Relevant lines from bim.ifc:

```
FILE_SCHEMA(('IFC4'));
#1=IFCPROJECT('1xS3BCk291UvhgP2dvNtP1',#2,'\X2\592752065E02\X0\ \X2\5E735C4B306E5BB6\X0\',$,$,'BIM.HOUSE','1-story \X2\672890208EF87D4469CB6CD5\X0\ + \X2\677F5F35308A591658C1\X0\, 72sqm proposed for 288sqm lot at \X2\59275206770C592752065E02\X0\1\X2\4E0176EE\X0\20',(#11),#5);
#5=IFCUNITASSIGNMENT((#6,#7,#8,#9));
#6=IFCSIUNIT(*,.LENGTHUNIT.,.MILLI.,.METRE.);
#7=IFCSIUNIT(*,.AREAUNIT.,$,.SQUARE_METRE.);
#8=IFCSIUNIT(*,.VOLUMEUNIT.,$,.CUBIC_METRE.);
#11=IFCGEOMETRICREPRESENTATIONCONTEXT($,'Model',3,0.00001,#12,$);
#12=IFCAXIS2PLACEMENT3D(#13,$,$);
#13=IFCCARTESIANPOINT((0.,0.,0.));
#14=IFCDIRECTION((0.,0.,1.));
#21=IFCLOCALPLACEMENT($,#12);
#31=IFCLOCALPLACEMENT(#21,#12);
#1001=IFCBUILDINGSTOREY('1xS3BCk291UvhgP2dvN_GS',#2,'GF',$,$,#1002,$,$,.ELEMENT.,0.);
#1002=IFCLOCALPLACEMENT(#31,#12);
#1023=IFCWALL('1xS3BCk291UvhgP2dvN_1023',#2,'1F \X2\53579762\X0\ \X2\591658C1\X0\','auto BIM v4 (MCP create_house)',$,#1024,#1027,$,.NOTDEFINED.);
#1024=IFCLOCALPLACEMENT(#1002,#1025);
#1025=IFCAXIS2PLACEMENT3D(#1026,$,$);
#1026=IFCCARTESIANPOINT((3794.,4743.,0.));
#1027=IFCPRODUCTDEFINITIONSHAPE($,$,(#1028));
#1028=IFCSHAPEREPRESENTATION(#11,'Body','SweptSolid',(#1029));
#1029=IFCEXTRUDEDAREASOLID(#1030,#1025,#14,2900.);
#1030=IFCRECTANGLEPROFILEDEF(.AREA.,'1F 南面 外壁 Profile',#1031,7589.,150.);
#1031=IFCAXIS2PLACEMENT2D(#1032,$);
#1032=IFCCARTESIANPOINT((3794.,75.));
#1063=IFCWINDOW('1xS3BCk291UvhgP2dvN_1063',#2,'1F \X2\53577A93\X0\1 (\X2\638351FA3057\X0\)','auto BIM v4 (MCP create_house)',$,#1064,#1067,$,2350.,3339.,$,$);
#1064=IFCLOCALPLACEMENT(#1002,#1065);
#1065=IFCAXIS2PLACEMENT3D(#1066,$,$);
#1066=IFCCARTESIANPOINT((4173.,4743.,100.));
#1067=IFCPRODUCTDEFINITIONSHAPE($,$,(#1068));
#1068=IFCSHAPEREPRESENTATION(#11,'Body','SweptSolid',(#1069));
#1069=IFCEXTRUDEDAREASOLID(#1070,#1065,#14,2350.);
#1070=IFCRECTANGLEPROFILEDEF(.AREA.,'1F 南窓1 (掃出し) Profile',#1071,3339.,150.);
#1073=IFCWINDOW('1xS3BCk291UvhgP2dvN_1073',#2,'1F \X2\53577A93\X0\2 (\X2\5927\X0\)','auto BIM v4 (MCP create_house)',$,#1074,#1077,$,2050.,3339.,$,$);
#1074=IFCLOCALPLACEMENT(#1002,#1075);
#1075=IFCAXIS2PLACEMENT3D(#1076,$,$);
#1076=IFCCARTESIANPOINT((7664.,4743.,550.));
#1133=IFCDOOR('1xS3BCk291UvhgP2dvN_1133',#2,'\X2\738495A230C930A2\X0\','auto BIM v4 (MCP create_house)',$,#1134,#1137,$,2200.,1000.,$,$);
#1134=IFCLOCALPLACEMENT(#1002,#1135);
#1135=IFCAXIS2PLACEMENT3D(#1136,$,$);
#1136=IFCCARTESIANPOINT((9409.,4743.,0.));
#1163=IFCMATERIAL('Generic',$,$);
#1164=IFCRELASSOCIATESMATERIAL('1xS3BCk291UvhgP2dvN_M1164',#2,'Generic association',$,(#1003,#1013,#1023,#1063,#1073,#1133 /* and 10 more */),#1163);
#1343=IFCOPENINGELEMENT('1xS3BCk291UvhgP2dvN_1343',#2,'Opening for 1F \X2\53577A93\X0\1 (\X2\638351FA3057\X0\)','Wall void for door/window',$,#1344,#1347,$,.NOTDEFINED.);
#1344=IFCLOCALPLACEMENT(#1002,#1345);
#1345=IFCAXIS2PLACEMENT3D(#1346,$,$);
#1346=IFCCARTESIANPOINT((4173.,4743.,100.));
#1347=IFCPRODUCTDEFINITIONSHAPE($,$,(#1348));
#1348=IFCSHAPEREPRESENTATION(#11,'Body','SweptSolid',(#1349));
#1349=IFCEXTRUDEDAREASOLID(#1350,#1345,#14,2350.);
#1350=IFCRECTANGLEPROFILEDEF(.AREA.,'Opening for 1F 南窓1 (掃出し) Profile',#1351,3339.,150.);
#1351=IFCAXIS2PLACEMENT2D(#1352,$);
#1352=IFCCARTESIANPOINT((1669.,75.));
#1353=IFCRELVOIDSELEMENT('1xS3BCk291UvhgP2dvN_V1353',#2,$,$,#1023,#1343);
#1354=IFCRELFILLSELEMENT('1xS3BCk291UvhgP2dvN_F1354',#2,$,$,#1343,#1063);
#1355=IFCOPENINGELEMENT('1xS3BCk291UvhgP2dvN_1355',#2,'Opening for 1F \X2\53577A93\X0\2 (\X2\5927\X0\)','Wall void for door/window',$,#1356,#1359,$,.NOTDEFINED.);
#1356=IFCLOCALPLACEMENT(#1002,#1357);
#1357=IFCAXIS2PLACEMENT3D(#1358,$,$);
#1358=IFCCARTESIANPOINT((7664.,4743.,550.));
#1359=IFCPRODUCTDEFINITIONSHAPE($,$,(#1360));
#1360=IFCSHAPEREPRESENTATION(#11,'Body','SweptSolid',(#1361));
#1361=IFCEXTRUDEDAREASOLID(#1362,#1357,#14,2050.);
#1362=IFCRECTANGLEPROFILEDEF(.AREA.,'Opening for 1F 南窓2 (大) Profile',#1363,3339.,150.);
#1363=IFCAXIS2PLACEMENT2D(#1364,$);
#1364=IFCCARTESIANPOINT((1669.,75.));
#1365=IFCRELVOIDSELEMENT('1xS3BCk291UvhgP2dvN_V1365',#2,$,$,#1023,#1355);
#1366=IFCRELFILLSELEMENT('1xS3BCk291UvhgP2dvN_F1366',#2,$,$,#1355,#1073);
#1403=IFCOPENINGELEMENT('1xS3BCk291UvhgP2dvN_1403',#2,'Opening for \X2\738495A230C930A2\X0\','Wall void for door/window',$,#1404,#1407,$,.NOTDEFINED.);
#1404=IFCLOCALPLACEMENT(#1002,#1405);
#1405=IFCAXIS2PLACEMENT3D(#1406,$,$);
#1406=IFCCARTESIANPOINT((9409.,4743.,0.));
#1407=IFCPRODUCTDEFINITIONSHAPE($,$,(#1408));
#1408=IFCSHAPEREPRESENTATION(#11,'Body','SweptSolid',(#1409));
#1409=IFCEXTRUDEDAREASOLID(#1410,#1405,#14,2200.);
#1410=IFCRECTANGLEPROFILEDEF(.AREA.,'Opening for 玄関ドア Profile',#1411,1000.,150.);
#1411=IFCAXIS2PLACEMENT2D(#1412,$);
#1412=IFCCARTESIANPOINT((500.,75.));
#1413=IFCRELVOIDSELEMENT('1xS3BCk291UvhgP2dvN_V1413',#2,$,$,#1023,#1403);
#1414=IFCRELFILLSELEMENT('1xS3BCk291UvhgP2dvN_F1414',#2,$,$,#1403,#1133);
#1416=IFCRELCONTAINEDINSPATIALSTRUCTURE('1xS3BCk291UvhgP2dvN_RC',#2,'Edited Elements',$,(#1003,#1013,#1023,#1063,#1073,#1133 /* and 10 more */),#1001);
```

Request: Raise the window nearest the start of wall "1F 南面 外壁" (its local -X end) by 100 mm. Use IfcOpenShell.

```python
import numpy as np
import ifcopenshell
import ifcopenshell.api.geometry
import ifcopenshell.util.placement
import ifcopenshell.util.unit

model = ifcopenshell.open("bim.ifc")
unit_scale = ifcopenshell.util.unit.calculate_unit_scale(model)

window = model.by_guid("1xS3BCk291UvhgP2dvN_1063")
opening = window.FillsVoids[0].RelatingOpeningElement
dz = 100.0

shift = np.array([0.0, 0.0, dz])
# The window is not placed relative to its opening, so move both.
for product in (opening, window):
    matrix = ifcopenshell.util.placement.get_local_placement(product.ObjectPlacement)
    matrix[:3, 3] += shift
    ifcopenshell.api.geometry.edit_object_placement(model, product=product, matrix=matrix, is_si=False)

print(f"moved by {dz * unit_scale:+.3f} m")

model.write("bim_v2.ifc")
```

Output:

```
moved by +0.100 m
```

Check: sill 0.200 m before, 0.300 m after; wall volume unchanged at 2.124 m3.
